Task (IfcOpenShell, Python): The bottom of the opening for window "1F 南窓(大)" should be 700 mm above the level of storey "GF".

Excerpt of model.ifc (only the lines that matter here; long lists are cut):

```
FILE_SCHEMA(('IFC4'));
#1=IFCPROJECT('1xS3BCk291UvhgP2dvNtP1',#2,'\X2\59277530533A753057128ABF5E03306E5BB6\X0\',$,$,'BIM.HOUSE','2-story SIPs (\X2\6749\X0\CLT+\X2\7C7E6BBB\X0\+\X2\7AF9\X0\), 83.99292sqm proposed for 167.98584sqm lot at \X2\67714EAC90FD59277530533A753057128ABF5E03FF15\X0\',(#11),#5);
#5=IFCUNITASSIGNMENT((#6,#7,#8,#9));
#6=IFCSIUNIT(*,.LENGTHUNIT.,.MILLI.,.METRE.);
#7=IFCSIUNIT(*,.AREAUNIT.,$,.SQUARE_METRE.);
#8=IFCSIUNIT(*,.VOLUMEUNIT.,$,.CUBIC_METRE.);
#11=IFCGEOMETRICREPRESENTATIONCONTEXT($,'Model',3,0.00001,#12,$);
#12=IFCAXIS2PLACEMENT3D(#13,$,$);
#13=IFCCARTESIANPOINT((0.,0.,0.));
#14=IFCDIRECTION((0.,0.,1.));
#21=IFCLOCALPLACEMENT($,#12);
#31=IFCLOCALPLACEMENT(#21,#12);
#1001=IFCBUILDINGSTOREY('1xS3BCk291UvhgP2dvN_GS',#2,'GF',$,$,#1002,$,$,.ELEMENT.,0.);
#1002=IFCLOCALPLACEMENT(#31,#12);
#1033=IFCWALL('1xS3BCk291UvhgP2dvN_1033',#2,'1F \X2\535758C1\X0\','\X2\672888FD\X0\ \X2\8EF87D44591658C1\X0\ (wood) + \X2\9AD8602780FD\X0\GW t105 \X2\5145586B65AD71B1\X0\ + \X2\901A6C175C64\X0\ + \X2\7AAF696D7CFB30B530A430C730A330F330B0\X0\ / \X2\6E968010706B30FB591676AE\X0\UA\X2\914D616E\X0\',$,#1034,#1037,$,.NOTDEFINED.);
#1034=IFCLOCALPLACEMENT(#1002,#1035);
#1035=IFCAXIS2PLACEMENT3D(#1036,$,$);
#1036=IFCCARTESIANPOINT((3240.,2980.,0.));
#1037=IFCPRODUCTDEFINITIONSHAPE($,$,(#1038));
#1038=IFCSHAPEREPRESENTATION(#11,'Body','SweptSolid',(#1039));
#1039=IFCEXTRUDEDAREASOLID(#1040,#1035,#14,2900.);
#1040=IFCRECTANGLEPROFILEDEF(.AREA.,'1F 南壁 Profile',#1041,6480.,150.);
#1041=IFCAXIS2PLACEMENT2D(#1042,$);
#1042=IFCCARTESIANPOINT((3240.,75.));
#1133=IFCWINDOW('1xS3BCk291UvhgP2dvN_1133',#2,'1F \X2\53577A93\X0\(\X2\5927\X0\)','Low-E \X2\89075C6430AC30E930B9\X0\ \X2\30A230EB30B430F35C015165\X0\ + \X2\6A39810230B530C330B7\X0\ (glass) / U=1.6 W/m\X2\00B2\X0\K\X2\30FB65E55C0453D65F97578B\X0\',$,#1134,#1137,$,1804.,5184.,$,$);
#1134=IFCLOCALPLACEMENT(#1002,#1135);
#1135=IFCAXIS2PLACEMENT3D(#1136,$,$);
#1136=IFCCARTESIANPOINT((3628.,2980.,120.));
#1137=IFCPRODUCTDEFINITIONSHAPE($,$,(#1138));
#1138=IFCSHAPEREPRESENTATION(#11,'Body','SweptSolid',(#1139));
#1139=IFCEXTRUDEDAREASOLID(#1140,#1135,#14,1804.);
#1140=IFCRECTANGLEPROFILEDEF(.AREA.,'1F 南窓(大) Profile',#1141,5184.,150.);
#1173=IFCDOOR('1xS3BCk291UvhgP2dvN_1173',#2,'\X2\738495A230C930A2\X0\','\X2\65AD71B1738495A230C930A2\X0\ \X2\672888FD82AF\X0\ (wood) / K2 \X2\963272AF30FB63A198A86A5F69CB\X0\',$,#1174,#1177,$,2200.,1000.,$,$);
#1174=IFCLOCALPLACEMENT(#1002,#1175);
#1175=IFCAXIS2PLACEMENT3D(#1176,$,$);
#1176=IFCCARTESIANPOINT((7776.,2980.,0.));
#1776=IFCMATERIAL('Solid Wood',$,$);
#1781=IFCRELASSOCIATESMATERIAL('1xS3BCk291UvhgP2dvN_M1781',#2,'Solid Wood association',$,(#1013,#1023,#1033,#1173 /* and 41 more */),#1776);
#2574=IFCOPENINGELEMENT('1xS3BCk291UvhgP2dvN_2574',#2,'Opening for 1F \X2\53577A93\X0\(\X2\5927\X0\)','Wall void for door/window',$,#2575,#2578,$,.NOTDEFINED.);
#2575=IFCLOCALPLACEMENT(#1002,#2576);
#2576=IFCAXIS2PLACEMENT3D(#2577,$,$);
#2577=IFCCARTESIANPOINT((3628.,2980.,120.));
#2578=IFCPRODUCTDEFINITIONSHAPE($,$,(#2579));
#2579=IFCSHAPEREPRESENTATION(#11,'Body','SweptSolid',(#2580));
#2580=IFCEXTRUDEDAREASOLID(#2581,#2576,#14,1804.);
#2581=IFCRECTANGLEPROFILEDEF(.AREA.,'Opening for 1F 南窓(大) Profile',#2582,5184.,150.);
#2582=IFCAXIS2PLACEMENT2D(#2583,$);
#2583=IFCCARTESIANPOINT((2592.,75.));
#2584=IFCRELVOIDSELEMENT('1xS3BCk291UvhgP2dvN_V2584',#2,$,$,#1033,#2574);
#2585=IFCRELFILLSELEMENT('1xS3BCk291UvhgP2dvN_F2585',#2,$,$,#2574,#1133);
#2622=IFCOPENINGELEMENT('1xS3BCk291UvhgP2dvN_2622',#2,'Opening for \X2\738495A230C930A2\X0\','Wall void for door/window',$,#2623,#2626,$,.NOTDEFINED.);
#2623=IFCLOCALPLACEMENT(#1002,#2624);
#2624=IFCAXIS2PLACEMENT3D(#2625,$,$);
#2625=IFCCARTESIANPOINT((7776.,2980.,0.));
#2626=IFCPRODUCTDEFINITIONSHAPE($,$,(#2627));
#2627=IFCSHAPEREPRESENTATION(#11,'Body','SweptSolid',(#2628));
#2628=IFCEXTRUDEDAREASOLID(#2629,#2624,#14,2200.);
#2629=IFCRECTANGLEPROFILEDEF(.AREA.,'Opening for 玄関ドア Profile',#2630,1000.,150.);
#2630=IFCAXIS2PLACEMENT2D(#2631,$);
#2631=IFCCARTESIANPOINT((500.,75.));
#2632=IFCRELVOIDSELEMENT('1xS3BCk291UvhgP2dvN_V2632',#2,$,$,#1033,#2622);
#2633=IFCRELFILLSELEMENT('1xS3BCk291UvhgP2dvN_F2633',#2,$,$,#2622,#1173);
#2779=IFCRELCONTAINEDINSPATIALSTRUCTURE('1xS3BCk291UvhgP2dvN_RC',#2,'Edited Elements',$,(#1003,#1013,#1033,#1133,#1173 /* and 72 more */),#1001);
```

```python
import numpy as np
import ifcopenshell
import ifcopenshell.api.geometry
import ifcopenshell.geom
import ifcopenshell.util.element
import ifcopenshell.util.placement
import ifcopenshell.util.shape
import ifcopenshell.util.unit

model = ifcopenshell.open("model.ifc")
unit_scale = ifcopenshell.util.unit.calculate_unit_scale(model)

window = model.by_guid("1xS3BCk291UvhgP2dvN_1133")
opening = window.FillsVoids[0].RelatingOpeningElement
storey = ifcopenshell.util.element.get_container(window, ifc_class="IfcBuildingStorey")
level = ifcopenshell.util.placement.get_local_placement(storey.ObjectPlacement)[2, 3]

# The opening's origin need not be at the sill, so measure its lowest point.
shape = ifcopenshell.geom.create_shape(ifcopenshell.geom.settings(), opening)
bottom = ifcopenshell.util.shape.get_shape_bottom_elevation(shape, shape.geometry) / unit_scale
dz = level + 0.7 / unit_scale - bottom

shift = np.array([0.0, 0.0, dz])
# The window is not placed relative to its opening, so move both.
for product in (opening, window):
    matrix = ifcopenshell.util.placement.get_local_placement(product.ObjectPlacement)
    matrix[:3, 3] += shift
    ifcopenshell.api.geometry.edit_object_placement(model, product=product, matrix=matrix, is_si=False)

print(f"moved by {dz * unit_scale:+.3f} m")

model.write("model_rev.ifc")
```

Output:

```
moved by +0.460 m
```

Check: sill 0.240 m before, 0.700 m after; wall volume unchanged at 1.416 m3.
